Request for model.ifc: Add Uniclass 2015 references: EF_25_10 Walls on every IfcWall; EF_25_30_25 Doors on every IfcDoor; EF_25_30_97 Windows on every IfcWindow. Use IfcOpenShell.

First a look at what the model holds.

```python
import ifcopenshell

model = ifcopenshell.open("model.ifc")
print(model.schema)
print("classifications:", [c.Name for c in model.by_type("IfcClassification")])
for ifc_class in ("IfcDoor", "IfcRoof", "IfcStair", "IfcWall", "IfcWindow"):
    print(ifc_class, len(model.by_type(ifc_class)))
```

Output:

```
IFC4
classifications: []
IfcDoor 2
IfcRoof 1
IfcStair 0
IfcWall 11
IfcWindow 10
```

```python
import ifcopenshell
import ifcopenshell.api.classification

model = ifcopenshell.open("model.ifc")

system = ifcopenshell.api.classification.add_classification(model, classification="Uniclass 2015")

codes = {
    "IfcWall": ("EF_25_10", "Walls"),
    "IfcDoor": ("EF_25_30_25", "Doors"),
    "IfcWindow": ("EF_25_30_97", "Windows"),
}
for ifc_class, (code, name) in codes.items():
    products = model.by_type(ifc_class)
    ifcopenshell.api.classification.add_reference(
        model, products=products, classification=system, identification=code, name=name
    )
    print(code, len(products))

model.write("model_v2.ifc")
```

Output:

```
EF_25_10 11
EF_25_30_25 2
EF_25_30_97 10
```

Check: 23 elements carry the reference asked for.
